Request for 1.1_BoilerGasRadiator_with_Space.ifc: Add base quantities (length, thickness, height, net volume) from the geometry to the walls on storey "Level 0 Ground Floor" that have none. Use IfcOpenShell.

First a look at what the model holds.

```python
import ifcopenshell
import ifcopenshell.util.element
import ifcopenshell.util.unit

model = ifcopenshell.open("1.1_BoilerGasRadiator_with_Space.ifc")
print(model.schema)
for unit_type in ("LENGTHUNIT", "AREAUNIT", "VOLUMEUNIT"):
    print(unit_type, ifcopenshell.util.unit.calculate_unit_scale(model, unit_type))
storey = next(s for s in model.by_type("IfcBuildingStorey") if s.Name == "Level 0 Ground Floor")
walls = [e for e in ifcopenshell.util.element.get_decomposition(storey) if e.is_a("IfcWall")]
for e in sorted(walls, key=lambda e: e.id()):
    print(e.id(), e.is_a(), e.Name, list(ifcopenshell.util.element.get_psets(e, qtos_only=True)), sep=" | ")
```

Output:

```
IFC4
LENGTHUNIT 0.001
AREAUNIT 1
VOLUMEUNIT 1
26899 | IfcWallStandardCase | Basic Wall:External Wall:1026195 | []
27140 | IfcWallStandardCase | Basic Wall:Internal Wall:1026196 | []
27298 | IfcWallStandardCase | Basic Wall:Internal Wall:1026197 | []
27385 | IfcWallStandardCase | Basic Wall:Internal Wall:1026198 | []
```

```python
import ifcopenshell
import ifcopenshell.api.pset
import ifcopenshell.geom
import ifcopenshell.util.element
import ifcopenshell.util.shape
import ifcopenshell.util.unit

model = ifcopenshell.open("1.1_BoilerGasRadiator_with_Space.ifc")
unit_scale = ifcopenshell.util.unit.calculate_unit_scale(model)
volume_scale = ifcopenshell.util.unit.calculate_unit_scale(model, "VOLUMEUNIT")
settings = ifcopenshell.geom.settings()

storey = next(s for s in model.by_type("IfcBuildingStorey") if s.Name == "Level 0 Ground Floor")
walls = [e for e in ifcopenshell.util.element.get_decomposition(storey) if e.is_a("IfcWall")]

for e in sorted(walls, key=lambda e: e.id()):
    if ifcopenshell.util.element.get_psets(e, qtos_only=True, should_inherit=False):
        continue
    # Geometry comes back in metres, in the element's own axes.
    shape = ifcopenshell.geom.create_shape(settings, e)
    values = {
        "Length": ifcopenshell.util.shape.get_x(shape.geometry) / unit_scale,
        "Width": ifcopenshell.util.shape.get_y(shape.geometry) / unit_scale,
        "Height": ifcopenshell.util.shape.get_z(shape.geometry) / unit_scale,
        "NetVolume": ifcopenshell.util.shape.get_volume(shape.geometry) / volume_scale,
    }
    qto = ifcopenshell.api.pset.add_qto(model, product=e, name="Qto_WallBaseQuantities")
    ifcopenshell.api.pset.edit_qto(model, qto=qto, properties=values)
    print(e.id(), {k: round(v, 3) for k, v in values.items()})

model.write("1.1_BoilerGasRadiator_with_Space_edited.ifc")
```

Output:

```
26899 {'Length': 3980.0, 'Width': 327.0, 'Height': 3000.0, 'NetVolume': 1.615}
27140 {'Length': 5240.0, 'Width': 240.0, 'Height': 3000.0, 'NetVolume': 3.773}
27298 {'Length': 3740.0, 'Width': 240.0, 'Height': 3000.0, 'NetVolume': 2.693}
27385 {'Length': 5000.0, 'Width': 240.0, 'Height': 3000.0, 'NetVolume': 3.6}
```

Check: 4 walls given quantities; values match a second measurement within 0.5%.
